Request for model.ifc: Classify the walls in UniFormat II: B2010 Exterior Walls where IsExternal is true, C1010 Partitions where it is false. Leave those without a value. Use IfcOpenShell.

First a look at what the model holds.

```python
import ifcopenshell
import ifcopenshell.util.element

model = ifcopenshell.open("model.ifc")
print(model.schema)
print("classifications:", [c.Name for c in model.by_type("IfcClassification")])
values = [ifcopenshell.util.element.get_pset(e, "Pset_WallCommon", "IsExternal") for e in model.by_type("IfcWall")]
for value in (True, False, None):
    print("IsExternal", value, values.count(value))
```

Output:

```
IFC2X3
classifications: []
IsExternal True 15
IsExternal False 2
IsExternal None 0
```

```python
import ifcopenshell
import ifcopenshell.api.classification
import ifcopenshell.util.element

model = ifcopenshell.open("model.ifc")

# IFC2X3 requires Source and Edition and has no link from the project to the system.
system = model.create_entity("IfcClassification", Source="ASTM", Edition="E1557", Name="UniFormat II")

walls = model.by_type("IfcWall")
external = {e: ifcopenshell.util.element.get_pset(e, "Pset_WallCommon", "IsExternal") for e in walls}
for flag, code, name in ((True, "B2010", "Exterior Walls"), (False, "C1010", "Partitions")):
    products = [e for e in walls if external[e] is flag]
    ifcopenshell.api.classification.add_reference(
        model, products=products, classification=system, identification=code, name=name
    )
    print(code, len(products))

model.write("model_updated.ifc")
```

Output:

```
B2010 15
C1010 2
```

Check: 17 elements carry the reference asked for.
